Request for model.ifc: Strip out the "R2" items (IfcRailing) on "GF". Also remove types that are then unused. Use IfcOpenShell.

First a look at what the model holds.

```python
import ifcopenshell
import ifcopenshell.util.element

model = ifcopenshell.open("model.ifc")
print(model.schema)
storey = next(s for s in model.by_type("IfcBuildingStorey") if s.Name == "GF")
railings = [e for e in ifcopenshell.util.element.get_decomposition(storey) if e.is_a("IfcRailing")]
seen = {}
for e in railings:
    element_type = ifcopenshell.util.element.get_type(e)
    name = element_type.Name if element_type not in (None, e) else None
    seen[name] = seen.get(name, 0) + 1
for name, count in sorted(seen.items(), key=str):
    print(count, "x", name)
```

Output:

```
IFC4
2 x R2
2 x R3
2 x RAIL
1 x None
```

```python
import ifcopenshell
import ifcopenshell.api.root
import ifcopenshell.util.element

model = ifcopenshell.open("model.ifc")

storey = next(s for s in model.by_type("IfcBuildingStorey") if s.Name == "GF")
railings = [e for e in ifcopenshell.util.element.get_decomposition(storey) if e.is_a("IfcRailing")]
targets = [e for e in railings if (t := ifcopenshell.util.element.get_type(e)) not in (None, e) and t.Name == "R2"]
types = {ifcopenshell.util.element.get_type(e) for e in targets} - {None, *targets}

for e in targets:
    ifcopenshell.api.root.remove_product(model, product=e)
print(len(targets), "removed")

unused = [t for t in types if not ifcopenshell.util.element.get_types(t)]
for t in unused:
    ifcopenshell.api.root.remove_product(model, product=t)
print(len(unused), "unused types removed")

model.write("model_updated.ifc")
```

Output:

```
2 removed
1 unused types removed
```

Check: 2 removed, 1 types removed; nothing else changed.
